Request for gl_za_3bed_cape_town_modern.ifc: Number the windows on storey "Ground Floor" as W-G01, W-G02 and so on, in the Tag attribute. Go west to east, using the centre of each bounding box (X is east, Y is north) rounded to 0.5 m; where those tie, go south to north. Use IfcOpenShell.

First a look at what the model holds.

```python
import ifcopenshell
import ifcopenshell.util.element
import ifcopenshell.util.placement

model = ifcopenshell.open("gl_za_3bed_cape_town_modern.ifc")
print(model.schema)
storey = next(s for s in model.by_type("IfcBuildingStorey") if s.Name == "Ground Floor")
windows = [e for e in ifcopenshell.util.element.get_decomposition(storey) if e.is_a("IfcWindow")]
for e in sorted(windows, key=lambda e: e.id()):
    origin = ifcopenshell.util.placement.get_local_placement(e.ObjectPlacement)[:3, 3]
    print(e.id(), e.Tag, e.Name, origin.round(2) + 0.0, sep=" | ")
```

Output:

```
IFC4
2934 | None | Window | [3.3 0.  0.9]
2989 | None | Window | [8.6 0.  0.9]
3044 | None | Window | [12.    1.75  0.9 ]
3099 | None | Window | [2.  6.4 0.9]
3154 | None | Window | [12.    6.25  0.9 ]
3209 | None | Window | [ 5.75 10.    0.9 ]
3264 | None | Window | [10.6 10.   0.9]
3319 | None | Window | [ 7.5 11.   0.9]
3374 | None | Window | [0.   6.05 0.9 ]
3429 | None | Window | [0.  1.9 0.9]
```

```python
import ifcopenshell
import ifcopenshell.geom
import ifcopenshell.util.element
import ifcopenshell.util.shape

model = ifcopenshell.open("gl_za_3bed_cape_town_modern.ifc")
settings = ifcopenshell.geom.settings()
settings.set("use-world-coords", True)


def centre(element):
    shape = ifcopenshell.geom.create_shape(settings, element)
    return ifcopenshell.util.shape.get_bbox_centroid(shape.geometry)


storey = next(s for s in model.by_type("IfcBuildingStorey") if s.Name == "Ground Floor")
windows = [e for e in ifcopenshell.util.element.get_decomposition(storey) if e.is_a("IfcWindow")]

# Insertion points can sit at a corner or the storey origin, so sort by the geometry (in metres).
centres = {e: centre(e) for e in windows}
windows.sort(key=lambda e: (round(centres[e][0] / 0.5), centres[e][1]))

for i, e in enumerate(windows, start=1):
    number = f"W-G{i:02d}"
    e.Tag = number
    print(e.id(), number)

model.write("gl_za_3bed_cape_town_modern_edited.ifc")
```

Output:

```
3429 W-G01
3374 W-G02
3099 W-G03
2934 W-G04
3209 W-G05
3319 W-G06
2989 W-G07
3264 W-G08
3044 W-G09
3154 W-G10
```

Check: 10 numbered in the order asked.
